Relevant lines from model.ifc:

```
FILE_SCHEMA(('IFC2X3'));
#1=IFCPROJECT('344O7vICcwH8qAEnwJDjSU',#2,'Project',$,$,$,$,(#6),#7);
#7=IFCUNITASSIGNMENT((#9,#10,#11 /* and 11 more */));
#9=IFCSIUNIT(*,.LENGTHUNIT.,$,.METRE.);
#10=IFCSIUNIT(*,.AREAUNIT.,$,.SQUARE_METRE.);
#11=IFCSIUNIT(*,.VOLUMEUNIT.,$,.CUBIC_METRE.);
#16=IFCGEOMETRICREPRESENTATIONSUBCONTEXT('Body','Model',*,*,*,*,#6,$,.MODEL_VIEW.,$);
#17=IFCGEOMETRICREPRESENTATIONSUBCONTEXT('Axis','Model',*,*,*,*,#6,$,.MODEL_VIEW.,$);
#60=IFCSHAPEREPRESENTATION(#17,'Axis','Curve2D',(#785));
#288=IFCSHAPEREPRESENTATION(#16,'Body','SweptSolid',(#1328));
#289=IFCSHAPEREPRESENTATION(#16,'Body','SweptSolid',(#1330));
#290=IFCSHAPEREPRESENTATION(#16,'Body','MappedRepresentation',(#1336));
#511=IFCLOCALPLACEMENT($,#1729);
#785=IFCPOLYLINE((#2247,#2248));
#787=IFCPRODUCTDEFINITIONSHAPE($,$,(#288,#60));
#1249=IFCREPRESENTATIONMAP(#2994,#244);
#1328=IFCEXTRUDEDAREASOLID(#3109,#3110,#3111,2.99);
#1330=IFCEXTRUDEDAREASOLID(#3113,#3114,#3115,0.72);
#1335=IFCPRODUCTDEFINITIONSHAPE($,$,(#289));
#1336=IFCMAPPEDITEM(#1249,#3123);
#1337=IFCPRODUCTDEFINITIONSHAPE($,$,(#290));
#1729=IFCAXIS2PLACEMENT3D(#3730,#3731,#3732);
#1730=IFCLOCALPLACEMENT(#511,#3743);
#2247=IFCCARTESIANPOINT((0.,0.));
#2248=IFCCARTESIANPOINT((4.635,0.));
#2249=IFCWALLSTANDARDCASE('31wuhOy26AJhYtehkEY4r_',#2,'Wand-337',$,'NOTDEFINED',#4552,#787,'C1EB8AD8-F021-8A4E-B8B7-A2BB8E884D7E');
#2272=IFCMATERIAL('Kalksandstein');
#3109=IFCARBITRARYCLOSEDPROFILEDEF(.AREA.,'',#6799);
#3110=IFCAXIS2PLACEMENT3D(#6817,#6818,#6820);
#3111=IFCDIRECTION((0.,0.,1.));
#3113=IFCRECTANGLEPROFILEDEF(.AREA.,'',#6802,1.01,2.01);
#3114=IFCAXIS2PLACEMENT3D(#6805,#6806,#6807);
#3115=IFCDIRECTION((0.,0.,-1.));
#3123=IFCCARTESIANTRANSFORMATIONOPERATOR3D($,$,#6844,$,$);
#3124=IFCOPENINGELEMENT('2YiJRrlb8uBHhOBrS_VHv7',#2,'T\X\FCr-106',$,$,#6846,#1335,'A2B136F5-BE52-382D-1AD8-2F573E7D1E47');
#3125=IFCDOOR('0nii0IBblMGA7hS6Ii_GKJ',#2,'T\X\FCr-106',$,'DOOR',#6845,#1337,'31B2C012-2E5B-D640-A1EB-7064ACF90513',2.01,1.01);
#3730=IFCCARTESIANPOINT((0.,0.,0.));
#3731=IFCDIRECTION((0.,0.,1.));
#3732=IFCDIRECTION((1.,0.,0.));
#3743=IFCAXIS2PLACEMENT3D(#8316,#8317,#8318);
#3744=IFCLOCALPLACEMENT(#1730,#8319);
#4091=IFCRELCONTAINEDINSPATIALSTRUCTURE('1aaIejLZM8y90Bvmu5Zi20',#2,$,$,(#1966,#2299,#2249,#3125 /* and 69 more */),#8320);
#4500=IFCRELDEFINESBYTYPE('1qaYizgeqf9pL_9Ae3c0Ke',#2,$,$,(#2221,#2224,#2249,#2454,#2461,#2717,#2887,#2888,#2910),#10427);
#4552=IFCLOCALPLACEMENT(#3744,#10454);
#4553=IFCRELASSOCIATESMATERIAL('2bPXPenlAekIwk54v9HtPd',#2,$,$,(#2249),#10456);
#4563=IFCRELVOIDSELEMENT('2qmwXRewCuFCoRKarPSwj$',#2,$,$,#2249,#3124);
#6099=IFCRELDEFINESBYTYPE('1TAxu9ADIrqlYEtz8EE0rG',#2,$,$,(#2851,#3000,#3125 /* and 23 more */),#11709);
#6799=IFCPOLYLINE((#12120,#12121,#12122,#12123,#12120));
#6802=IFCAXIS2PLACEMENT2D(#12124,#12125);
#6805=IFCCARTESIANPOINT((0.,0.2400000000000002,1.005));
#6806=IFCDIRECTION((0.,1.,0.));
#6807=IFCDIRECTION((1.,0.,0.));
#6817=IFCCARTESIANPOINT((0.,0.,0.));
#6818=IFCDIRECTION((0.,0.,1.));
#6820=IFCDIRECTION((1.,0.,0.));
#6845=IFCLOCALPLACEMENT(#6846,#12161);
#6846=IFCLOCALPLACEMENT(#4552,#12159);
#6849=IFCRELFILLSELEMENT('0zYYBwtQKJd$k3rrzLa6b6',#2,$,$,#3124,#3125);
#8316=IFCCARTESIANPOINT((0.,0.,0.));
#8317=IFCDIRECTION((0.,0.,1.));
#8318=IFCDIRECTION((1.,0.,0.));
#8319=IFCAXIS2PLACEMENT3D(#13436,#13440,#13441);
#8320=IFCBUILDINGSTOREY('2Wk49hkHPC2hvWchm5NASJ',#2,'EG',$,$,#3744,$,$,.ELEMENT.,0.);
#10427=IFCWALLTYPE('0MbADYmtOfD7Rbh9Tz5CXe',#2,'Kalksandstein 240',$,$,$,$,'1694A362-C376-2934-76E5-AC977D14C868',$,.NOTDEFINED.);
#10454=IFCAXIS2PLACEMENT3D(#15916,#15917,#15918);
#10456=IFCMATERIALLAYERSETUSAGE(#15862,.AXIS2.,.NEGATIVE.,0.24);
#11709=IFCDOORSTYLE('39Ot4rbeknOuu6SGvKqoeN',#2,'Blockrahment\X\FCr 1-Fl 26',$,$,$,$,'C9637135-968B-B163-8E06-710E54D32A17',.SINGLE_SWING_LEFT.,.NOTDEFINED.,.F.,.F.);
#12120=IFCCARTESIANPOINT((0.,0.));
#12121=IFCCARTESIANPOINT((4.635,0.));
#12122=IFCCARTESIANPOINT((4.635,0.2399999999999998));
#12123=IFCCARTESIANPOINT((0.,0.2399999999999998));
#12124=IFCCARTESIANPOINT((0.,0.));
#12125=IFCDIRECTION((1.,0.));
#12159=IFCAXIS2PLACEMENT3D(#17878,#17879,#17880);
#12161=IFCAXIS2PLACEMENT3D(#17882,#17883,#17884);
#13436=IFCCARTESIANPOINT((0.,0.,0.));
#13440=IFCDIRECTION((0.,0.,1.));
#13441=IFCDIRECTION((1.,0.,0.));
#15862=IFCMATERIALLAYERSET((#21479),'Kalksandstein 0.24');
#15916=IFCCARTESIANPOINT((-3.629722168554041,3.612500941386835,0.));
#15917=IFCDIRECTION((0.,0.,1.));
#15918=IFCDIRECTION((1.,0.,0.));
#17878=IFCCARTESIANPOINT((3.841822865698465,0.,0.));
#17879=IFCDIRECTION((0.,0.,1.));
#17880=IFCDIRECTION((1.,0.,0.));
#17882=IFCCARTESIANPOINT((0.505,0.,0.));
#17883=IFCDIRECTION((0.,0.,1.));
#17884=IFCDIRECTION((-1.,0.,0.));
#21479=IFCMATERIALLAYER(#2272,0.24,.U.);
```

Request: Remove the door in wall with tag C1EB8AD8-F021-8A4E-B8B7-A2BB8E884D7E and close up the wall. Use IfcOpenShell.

```python
import ifcopenshell
import ifcopenshell.api.feature
import ifcopenshell.api.root
import ifcopenshell.geom
import ifcopenshell.util.shape

model = ifcopenshell.open("model.ifc")
settings = ifcopenshell.geom.settings()


def volume(element):
    """Net volume in cubic metres, openings subtracted."""
    shape = ifcopenshell.geom.create_shape(settings, element)
    return ifcopenshell.util.shape.get_volume(shape.geometry)


door = model.by_guid("0nii0IBblMGA7hS6Ii_GKJ")
opening = door.FillsVoids[0].RelatingOpeningElement
wall = opening.VoidsElements[0].RelatingBuildingElement
before = volume(wall)

ifcopenshell.api.root.remove_product(model, product=door)
ifcopenshell.api.feature.remove_feature(model, feature=opening)

after = volume(wall)

print(f"wall volume {before:.3f} -> {after:.3f} m3")

model.write("model_updated.ifc")
```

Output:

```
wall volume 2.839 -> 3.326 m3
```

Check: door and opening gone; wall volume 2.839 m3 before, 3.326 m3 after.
